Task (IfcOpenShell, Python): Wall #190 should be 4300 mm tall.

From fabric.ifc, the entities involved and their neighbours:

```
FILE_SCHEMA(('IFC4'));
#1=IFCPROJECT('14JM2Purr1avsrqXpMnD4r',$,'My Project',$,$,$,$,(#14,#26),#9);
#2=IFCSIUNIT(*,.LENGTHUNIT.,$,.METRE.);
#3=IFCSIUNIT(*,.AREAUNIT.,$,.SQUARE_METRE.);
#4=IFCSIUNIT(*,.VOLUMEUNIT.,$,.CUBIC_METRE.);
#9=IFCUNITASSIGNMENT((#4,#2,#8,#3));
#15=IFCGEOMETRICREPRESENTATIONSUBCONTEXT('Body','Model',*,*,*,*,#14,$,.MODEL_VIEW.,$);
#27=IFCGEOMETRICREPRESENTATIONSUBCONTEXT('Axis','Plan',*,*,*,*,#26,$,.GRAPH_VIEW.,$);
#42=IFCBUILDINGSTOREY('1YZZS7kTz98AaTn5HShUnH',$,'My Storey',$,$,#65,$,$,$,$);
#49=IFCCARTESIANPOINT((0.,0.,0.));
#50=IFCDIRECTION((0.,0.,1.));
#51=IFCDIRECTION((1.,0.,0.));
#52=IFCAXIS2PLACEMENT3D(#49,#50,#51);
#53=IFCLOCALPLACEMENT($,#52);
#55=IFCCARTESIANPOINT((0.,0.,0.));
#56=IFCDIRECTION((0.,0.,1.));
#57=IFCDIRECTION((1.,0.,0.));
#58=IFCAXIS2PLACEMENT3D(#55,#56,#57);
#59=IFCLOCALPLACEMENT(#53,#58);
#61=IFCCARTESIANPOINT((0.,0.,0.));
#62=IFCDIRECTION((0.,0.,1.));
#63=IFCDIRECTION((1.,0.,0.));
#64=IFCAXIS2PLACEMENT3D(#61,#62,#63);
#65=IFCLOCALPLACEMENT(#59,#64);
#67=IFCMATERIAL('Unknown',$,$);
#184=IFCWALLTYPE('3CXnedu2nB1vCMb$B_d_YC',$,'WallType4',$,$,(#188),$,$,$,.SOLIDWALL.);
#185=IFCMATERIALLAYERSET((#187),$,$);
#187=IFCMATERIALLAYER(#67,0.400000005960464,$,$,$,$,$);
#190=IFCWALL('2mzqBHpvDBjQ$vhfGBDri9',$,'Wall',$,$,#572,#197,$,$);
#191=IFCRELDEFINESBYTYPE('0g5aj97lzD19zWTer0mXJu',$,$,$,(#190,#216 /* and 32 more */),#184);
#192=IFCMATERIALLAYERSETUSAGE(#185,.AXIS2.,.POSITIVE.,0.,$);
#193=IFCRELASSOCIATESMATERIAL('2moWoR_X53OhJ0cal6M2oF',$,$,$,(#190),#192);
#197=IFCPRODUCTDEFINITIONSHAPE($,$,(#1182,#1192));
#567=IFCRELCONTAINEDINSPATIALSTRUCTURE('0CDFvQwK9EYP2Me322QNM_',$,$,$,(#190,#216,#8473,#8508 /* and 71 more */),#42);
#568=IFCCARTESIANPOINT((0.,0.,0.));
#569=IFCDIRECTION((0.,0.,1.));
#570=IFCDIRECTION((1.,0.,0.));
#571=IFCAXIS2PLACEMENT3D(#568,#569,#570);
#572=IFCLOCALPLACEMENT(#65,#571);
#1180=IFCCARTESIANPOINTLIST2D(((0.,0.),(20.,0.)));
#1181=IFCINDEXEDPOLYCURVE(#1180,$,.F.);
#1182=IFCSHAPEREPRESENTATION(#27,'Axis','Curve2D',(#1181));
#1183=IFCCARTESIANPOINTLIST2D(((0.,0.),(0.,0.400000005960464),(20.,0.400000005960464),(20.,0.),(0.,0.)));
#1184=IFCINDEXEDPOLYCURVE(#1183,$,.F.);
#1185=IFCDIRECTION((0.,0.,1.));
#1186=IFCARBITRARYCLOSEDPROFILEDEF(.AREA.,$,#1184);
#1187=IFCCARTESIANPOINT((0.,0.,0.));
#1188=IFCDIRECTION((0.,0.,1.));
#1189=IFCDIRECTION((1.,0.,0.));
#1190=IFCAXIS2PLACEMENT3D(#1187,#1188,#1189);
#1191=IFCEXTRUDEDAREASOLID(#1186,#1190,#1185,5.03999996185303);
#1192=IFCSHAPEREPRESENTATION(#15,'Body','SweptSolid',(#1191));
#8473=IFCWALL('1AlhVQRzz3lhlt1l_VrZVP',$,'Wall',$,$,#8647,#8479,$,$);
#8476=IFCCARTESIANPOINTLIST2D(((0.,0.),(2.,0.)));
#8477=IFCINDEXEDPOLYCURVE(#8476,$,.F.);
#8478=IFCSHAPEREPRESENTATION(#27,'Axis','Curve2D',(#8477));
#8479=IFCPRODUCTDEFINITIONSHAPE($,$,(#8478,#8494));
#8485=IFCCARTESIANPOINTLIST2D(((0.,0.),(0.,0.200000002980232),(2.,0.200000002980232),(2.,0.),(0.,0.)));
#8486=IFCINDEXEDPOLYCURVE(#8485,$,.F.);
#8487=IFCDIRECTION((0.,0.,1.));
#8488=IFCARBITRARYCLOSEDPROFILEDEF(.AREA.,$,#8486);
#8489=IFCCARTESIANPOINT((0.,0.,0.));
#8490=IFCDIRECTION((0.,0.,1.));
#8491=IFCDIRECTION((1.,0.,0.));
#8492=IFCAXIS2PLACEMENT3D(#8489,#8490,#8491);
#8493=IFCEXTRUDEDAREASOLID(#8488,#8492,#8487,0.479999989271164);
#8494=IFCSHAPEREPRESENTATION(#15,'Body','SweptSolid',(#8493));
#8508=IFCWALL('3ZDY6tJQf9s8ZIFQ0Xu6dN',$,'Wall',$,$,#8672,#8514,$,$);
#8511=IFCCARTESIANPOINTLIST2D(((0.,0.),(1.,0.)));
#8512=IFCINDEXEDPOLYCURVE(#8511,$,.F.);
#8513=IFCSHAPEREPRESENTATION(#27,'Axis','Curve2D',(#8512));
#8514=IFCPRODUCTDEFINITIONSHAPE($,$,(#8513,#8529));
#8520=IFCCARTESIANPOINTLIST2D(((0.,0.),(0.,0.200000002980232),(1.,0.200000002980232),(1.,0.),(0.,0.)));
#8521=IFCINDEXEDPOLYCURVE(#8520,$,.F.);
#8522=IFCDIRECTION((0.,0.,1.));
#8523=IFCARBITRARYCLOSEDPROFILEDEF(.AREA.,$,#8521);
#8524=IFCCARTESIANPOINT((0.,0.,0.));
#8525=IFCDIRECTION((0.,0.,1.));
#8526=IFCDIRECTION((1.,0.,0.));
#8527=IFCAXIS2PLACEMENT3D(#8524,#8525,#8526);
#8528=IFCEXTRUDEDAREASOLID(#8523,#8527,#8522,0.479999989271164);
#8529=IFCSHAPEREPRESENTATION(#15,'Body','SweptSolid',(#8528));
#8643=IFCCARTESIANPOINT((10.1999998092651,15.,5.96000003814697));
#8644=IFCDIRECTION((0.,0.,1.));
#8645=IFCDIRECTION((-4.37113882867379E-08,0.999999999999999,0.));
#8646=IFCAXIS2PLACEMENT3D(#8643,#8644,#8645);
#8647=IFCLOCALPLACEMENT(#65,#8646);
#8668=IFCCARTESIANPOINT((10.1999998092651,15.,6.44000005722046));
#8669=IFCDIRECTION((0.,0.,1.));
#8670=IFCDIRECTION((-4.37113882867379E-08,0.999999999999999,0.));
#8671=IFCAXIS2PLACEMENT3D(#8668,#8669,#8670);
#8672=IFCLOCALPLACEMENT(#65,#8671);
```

```python
import ifcopenshell
import ifcopenshell.geom
import ifcopenshell.util.representation
import ifcopenshell.util.shape

model = ifcopenshell.open("fabric.ifc")
settings = ifcopenshell.geom.settings()


def volume(element):
    """Net volume in cubic metres, openings subtracted."""
    shape = ifcopenshell.geom.create_shape(settings, element)
    return ifcopenshell.util.shape.get_volume(shape.geometry)


wall = model.by_id(190)
before = volume(wall)

body = ifcopenshell.util.representation.get_representation(wall, "Model", "Body")
solid = body.Items[0]
old_height = solid.Depth
solid.Depth = 4.3
after = volume(wall)

print(f"height {old_height:g} -> {solid.Depth:g}, volume {before:.3f} -> {after:.3f} m3")

model.write("fabric_updated.ifc")
```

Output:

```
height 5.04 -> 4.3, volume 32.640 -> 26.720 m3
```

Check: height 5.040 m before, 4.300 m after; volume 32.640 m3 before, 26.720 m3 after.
